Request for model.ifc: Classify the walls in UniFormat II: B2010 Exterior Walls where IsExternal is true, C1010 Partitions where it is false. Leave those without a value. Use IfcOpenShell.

First a look at what the model holds.

```python
import ifcopenshell
import ifcopenshell.util.element

model = ifcopenshell.open("model.ifc")
print(model.schema)
print("classifications:", [c.Name for c in model.by_type("IfcClassification")])
values = [ifcopenshell.util.element.get_pset(e, "Pset_WallCommon", "IsExternal") for e in model.by_type("IfcWall")]
for value in (True, False, None):
    print("IsExternal", value, values.count(value))
```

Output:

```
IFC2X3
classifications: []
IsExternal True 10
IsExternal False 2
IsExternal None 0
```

```python
import ifcopenshell
import ifcopenshell.api.classification
import ifcopenshell.util.element

model = ifcopenshell.open("model.ifc")

# IFC2X3 requires Source and Edition and has no link from the project to the system.
system = model.create_entity("IfcClassification", Source="ASTM", Edition="E1557", Name="UniFormat II")

walls = model.by_type("IfcWall")
external = {e: ifcopenshell.util.element.get_pset(e, "Pset_WallCommon", "IsExternal") for e in walls}
for flag, code, name in ((True, "B2010", "Exterior Walls"), (False, "C1010", "Partitions")):
    products = [e for e in walls if external[e] is flag]
    ifcopenshell.api.classification.add_reference(
        model, products=products, classification=system, identification=code, name=name
    )
    print(code, len(products))

model.write("model-out.ifc")
```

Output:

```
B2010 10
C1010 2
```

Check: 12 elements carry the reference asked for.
